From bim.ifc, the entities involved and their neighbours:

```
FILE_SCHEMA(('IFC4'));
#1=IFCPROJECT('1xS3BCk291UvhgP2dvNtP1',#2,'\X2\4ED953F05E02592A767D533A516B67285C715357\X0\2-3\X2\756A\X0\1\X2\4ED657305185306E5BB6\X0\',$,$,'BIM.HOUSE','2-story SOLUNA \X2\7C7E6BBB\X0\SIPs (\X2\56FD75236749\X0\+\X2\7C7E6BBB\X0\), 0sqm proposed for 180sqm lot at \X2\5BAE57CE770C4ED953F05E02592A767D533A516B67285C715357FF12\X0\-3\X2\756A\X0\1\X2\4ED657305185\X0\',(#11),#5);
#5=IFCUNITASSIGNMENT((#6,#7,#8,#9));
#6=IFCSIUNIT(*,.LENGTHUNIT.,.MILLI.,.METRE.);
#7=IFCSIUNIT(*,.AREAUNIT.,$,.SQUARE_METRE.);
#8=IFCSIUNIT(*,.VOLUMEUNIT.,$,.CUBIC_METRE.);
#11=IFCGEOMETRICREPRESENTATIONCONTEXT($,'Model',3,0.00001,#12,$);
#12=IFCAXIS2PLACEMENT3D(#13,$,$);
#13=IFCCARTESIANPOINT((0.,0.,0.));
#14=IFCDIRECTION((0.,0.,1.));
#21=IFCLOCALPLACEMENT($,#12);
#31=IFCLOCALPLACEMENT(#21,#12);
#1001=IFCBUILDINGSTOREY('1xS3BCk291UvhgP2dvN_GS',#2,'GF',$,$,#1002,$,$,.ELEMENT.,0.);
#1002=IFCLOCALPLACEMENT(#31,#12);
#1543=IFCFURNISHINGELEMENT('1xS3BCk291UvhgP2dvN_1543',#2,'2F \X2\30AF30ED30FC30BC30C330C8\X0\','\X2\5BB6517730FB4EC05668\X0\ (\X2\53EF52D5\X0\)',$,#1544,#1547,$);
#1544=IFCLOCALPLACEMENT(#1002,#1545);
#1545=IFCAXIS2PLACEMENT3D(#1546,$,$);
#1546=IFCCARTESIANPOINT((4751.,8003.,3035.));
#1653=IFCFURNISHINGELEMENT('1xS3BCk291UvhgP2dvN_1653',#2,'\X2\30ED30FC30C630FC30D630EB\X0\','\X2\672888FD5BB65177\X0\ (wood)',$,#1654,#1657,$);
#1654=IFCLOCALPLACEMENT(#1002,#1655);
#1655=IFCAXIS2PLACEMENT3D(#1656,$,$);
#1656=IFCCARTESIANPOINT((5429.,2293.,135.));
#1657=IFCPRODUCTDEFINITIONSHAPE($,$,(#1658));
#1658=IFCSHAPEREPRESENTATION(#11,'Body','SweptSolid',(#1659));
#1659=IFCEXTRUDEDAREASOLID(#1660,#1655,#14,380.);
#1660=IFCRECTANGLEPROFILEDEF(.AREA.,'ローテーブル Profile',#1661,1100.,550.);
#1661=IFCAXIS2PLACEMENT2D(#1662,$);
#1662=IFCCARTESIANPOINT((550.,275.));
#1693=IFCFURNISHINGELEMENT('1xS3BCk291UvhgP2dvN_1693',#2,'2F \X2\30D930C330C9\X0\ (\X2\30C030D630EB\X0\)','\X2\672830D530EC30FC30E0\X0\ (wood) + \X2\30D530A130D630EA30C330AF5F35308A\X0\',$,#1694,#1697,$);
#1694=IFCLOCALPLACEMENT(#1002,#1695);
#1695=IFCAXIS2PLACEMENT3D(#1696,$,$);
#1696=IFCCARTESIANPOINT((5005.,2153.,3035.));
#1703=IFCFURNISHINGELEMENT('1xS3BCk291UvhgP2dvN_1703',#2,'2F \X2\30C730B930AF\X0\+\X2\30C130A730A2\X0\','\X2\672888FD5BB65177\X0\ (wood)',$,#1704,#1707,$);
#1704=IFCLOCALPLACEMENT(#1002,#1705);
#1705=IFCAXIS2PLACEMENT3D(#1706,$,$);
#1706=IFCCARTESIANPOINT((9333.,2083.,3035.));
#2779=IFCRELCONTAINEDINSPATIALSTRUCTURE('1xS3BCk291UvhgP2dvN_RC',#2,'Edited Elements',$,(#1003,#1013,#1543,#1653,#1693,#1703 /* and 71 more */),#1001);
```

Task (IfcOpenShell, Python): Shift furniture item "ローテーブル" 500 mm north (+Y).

```python
import ifcopenshell
import ifcopenshell.api.geometry
import ifcopenshell.util.placement
import ifcopenshell.util.unit

model = ifcopenshell.open("bim.ifc")
unit_scale = ifcopenshell.util.unit.calculate_unit_scale(model)

item = model.by_guid("1xS3BCk291UvhgP2dvN_1653")
matrix = ifcopenshell.util.placement.get_local_placement(item.ObjectPlacement)
matrix[1, 3] += 0.5 / unit_scale
ifcopenshell.api.geometry.edit_object_placement(model, product=item, matrix=matrix, is_si=False)

print(ifcopenshell.util.placement.get_local_placement(item.ObjectPlacement).round(3) + 0.0)

model.write("bim_v2.ifc")
```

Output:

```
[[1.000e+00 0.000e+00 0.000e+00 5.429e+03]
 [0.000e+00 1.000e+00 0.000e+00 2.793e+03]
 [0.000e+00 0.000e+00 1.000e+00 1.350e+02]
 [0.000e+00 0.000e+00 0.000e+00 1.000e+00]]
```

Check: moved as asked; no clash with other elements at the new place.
